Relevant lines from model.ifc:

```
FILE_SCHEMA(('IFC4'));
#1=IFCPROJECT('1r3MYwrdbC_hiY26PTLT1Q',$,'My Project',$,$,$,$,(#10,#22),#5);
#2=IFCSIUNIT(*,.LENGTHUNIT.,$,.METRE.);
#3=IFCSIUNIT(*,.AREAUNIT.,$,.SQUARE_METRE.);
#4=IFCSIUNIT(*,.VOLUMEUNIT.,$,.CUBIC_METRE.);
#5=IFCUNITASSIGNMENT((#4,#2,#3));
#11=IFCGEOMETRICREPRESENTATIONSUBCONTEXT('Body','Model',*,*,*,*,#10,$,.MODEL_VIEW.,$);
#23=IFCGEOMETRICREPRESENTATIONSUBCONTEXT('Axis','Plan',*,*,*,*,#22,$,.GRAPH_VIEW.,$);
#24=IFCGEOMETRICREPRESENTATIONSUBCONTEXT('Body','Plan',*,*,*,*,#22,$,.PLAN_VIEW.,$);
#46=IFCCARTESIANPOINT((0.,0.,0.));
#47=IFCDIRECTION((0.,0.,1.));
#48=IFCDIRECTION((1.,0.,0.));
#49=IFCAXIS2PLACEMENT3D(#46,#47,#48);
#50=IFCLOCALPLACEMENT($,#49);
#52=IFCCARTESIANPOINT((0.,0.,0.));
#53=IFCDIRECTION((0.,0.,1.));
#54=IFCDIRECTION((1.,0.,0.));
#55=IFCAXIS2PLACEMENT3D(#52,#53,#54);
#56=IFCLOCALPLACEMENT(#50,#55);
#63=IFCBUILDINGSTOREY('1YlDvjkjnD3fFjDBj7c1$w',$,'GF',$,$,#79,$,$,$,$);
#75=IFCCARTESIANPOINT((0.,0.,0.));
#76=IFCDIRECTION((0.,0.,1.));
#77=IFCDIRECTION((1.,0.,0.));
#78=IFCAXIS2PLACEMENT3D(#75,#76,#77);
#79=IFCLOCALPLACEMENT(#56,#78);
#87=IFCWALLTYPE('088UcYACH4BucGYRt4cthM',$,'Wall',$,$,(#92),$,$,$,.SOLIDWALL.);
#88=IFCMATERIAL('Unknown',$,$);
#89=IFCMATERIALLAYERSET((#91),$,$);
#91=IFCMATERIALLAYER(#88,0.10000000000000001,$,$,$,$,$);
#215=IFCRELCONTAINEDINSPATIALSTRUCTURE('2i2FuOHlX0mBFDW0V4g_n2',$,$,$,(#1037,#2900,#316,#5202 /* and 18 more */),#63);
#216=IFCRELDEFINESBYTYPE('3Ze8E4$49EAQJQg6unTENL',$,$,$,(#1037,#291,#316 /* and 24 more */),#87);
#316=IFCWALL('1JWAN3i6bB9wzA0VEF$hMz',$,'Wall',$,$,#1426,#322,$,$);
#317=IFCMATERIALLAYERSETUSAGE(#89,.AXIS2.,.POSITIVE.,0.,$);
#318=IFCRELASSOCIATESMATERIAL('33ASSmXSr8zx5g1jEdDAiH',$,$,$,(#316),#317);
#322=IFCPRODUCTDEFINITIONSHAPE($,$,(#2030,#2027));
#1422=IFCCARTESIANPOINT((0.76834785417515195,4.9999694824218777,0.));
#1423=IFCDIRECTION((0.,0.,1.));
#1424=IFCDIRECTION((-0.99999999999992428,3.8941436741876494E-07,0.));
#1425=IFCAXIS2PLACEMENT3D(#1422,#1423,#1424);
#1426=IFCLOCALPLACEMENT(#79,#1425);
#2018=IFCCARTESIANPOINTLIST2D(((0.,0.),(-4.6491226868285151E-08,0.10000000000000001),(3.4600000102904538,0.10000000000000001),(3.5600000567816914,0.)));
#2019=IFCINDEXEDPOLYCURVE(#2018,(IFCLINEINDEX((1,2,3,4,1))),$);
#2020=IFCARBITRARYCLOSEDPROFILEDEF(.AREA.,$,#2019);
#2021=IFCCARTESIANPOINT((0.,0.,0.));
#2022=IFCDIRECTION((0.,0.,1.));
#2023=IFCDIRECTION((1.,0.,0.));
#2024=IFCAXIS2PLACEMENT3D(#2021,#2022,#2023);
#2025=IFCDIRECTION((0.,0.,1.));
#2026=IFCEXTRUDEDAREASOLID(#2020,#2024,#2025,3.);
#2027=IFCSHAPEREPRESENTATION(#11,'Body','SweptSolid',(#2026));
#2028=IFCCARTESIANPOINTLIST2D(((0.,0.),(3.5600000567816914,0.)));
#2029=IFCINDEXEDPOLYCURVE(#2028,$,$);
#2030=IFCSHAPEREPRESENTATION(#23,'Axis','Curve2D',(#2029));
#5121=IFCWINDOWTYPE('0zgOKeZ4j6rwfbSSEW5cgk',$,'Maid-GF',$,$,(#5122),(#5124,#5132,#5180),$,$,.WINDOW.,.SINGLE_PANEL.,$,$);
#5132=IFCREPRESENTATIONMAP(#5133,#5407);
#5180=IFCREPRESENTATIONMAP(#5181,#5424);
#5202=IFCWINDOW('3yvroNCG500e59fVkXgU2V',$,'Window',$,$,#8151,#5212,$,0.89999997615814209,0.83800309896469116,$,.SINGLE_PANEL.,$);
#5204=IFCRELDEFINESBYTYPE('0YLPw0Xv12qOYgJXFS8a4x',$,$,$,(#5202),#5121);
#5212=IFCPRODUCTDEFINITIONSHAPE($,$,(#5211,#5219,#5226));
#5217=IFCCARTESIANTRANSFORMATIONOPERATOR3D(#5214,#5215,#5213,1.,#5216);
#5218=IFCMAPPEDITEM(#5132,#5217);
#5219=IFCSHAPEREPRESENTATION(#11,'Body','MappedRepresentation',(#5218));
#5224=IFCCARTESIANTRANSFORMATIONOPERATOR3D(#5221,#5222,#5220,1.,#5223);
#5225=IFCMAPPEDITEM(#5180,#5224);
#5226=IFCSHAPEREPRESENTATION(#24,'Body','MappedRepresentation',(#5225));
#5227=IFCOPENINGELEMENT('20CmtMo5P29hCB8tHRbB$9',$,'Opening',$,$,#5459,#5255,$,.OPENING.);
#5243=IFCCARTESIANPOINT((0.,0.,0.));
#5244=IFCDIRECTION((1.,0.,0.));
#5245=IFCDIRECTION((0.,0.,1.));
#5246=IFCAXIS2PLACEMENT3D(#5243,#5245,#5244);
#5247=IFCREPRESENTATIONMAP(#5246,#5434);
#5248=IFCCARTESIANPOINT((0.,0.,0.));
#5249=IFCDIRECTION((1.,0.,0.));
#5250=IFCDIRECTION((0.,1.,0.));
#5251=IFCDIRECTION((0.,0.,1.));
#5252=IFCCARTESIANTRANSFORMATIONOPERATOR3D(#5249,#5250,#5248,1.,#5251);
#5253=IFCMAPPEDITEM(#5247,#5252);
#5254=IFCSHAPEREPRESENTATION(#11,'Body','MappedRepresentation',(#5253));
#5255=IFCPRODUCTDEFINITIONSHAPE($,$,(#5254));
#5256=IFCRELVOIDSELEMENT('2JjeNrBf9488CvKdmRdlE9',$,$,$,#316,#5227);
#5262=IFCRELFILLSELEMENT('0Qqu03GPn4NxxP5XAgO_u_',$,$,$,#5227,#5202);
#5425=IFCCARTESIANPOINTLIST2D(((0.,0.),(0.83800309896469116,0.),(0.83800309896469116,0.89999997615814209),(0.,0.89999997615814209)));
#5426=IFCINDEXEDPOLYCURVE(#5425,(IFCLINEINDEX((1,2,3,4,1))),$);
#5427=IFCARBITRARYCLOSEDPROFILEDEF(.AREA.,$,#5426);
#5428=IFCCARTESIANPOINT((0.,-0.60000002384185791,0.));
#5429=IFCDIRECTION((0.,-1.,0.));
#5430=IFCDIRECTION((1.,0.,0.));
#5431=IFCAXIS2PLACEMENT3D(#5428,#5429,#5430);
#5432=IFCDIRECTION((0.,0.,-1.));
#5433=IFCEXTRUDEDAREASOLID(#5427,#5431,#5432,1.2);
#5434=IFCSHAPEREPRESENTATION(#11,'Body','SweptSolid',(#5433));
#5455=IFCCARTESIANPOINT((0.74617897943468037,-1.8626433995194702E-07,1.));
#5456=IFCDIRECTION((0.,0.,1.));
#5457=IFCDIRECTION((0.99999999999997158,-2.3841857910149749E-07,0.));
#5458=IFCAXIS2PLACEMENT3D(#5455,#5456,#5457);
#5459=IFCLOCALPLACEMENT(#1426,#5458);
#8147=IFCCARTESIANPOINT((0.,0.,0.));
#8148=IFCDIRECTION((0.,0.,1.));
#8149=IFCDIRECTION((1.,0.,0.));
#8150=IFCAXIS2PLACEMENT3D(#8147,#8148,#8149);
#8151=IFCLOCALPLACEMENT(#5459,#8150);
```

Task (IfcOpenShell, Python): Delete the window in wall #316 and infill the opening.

```python
import ifcopenshell
import ifcopenshell.api.feature
import ifcopenshell.api.root
import ifcopenshell.geom
import ifcopenshell.util.shape

model = ifcopenshell.open("model.ifc")
settings = ifcopenshell.geom.settings()


def volume(element):
    """Net volume in cubic metres, openings subtracted."""
    shape = ifcopenshell.geom.create_shape(settings, element)
    return ifcopenshell.util.shape.get_volume(shape.geometry)


window = model.by_guid("3yvroNCG500e59fVkXgU2V")
opening = window.FillsVoids[0].RelatingOpeningElement
wall = opening.VoidsElements[0].RelatingBuildingElement
before = volume(wall)

ifcopenshell.api.root.remove_product(model, product=window)
ifcopenshell.api.feature.remove_feature(model, feature=opening)

after = volume(wall)

print(f"wall volume {before:.3f} -> {after:.3f} m3")

model.write("model-out.ifc")
```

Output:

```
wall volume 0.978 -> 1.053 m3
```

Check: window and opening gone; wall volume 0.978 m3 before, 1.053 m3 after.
